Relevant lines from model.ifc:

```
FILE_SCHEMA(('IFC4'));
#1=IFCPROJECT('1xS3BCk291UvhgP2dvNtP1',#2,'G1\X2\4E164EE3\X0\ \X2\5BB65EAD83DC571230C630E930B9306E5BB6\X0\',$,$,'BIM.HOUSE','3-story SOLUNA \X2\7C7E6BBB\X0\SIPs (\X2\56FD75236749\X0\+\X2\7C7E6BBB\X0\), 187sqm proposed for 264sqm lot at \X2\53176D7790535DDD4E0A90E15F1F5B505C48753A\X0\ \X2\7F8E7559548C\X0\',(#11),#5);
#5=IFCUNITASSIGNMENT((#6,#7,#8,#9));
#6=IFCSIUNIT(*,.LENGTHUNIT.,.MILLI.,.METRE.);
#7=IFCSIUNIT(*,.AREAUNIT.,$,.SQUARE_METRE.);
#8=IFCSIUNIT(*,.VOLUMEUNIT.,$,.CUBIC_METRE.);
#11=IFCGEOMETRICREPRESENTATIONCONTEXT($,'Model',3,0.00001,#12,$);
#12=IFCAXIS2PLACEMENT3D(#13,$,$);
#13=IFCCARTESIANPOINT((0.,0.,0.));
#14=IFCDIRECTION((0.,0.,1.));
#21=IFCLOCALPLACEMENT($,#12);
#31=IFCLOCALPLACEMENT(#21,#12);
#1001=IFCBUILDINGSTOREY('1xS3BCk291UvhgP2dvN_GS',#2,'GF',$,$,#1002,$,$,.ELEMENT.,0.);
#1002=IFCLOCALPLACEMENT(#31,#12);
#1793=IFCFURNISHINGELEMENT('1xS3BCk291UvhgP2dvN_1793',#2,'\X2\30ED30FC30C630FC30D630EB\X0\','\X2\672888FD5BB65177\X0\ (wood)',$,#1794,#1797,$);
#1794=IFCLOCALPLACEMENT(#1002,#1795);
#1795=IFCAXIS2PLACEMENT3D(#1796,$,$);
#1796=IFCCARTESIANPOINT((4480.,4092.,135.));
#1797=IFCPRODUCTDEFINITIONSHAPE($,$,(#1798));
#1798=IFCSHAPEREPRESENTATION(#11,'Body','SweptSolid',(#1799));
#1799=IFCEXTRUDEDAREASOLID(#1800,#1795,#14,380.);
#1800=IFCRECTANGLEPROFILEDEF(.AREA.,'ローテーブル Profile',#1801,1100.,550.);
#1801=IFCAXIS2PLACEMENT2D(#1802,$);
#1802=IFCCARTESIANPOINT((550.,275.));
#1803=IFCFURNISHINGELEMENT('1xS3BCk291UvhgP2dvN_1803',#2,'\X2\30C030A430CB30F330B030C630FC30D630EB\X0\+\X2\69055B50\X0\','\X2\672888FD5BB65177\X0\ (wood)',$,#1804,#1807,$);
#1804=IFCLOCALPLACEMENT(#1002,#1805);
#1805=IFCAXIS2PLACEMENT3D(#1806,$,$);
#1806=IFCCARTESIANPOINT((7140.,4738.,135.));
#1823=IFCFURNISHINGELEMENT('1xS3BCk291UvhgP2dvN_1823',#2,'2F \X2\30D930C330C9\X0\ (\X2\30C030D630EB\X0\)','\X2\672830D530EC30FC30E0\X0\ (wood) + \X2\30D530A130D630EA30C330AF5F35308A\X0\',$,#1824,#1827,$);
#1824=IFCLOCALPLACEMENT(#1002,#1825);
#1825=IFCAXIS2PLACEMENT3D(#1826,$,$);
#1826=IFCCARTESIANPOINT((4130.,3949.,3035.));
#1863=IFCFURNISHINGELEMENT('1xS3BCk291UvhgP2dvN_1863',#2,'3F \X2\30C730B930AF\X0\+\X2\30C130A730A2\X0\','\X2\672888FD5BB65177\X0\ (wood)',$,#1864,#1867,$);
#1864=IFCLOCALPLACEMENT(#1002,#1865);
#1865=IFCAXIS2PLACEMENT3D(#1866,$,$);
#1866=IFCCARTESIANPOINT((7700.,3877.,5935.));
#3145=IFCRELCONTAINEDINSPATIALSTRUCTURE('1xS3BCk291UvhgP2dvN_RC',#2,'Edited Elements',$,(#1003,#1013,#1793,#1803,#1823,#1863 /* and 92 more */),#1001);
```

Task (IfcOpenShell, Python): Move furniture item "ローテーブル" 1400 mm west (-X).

```python
import ifcopenshell
import ifcopenshell.api.geometry
import ifcopenshell.util.placement
import ifcopenshell.util.unit

model = ifcopenshell.open("model.ifc")
unit_scale = ifcopenshell.util.unit.calculate_unit_scale(model)

item = model.by_id(1793)
matrix = ifcopenshell.util.placement.get_local_placement(item.ObjectPlacement)
matrix[0, 3] -= 1.4 / unit_scale
ifcopenshell.api.geometry.edit_object_placement(model, product=item, matrix=matrix, is_si=False)

print(ifcopenshell.util.placement.get_local_placement(item.ObjectPlacement).round(3) + 0.0)

model.write("model_edited.ifc")
```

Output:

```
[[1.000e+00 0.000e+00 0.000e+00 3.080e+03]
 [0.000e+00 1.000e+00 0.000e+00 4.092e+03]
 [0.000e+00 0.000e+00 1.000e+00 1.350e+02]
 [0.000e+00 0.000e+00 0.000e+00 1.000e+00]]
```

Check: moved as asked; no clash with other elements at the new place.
